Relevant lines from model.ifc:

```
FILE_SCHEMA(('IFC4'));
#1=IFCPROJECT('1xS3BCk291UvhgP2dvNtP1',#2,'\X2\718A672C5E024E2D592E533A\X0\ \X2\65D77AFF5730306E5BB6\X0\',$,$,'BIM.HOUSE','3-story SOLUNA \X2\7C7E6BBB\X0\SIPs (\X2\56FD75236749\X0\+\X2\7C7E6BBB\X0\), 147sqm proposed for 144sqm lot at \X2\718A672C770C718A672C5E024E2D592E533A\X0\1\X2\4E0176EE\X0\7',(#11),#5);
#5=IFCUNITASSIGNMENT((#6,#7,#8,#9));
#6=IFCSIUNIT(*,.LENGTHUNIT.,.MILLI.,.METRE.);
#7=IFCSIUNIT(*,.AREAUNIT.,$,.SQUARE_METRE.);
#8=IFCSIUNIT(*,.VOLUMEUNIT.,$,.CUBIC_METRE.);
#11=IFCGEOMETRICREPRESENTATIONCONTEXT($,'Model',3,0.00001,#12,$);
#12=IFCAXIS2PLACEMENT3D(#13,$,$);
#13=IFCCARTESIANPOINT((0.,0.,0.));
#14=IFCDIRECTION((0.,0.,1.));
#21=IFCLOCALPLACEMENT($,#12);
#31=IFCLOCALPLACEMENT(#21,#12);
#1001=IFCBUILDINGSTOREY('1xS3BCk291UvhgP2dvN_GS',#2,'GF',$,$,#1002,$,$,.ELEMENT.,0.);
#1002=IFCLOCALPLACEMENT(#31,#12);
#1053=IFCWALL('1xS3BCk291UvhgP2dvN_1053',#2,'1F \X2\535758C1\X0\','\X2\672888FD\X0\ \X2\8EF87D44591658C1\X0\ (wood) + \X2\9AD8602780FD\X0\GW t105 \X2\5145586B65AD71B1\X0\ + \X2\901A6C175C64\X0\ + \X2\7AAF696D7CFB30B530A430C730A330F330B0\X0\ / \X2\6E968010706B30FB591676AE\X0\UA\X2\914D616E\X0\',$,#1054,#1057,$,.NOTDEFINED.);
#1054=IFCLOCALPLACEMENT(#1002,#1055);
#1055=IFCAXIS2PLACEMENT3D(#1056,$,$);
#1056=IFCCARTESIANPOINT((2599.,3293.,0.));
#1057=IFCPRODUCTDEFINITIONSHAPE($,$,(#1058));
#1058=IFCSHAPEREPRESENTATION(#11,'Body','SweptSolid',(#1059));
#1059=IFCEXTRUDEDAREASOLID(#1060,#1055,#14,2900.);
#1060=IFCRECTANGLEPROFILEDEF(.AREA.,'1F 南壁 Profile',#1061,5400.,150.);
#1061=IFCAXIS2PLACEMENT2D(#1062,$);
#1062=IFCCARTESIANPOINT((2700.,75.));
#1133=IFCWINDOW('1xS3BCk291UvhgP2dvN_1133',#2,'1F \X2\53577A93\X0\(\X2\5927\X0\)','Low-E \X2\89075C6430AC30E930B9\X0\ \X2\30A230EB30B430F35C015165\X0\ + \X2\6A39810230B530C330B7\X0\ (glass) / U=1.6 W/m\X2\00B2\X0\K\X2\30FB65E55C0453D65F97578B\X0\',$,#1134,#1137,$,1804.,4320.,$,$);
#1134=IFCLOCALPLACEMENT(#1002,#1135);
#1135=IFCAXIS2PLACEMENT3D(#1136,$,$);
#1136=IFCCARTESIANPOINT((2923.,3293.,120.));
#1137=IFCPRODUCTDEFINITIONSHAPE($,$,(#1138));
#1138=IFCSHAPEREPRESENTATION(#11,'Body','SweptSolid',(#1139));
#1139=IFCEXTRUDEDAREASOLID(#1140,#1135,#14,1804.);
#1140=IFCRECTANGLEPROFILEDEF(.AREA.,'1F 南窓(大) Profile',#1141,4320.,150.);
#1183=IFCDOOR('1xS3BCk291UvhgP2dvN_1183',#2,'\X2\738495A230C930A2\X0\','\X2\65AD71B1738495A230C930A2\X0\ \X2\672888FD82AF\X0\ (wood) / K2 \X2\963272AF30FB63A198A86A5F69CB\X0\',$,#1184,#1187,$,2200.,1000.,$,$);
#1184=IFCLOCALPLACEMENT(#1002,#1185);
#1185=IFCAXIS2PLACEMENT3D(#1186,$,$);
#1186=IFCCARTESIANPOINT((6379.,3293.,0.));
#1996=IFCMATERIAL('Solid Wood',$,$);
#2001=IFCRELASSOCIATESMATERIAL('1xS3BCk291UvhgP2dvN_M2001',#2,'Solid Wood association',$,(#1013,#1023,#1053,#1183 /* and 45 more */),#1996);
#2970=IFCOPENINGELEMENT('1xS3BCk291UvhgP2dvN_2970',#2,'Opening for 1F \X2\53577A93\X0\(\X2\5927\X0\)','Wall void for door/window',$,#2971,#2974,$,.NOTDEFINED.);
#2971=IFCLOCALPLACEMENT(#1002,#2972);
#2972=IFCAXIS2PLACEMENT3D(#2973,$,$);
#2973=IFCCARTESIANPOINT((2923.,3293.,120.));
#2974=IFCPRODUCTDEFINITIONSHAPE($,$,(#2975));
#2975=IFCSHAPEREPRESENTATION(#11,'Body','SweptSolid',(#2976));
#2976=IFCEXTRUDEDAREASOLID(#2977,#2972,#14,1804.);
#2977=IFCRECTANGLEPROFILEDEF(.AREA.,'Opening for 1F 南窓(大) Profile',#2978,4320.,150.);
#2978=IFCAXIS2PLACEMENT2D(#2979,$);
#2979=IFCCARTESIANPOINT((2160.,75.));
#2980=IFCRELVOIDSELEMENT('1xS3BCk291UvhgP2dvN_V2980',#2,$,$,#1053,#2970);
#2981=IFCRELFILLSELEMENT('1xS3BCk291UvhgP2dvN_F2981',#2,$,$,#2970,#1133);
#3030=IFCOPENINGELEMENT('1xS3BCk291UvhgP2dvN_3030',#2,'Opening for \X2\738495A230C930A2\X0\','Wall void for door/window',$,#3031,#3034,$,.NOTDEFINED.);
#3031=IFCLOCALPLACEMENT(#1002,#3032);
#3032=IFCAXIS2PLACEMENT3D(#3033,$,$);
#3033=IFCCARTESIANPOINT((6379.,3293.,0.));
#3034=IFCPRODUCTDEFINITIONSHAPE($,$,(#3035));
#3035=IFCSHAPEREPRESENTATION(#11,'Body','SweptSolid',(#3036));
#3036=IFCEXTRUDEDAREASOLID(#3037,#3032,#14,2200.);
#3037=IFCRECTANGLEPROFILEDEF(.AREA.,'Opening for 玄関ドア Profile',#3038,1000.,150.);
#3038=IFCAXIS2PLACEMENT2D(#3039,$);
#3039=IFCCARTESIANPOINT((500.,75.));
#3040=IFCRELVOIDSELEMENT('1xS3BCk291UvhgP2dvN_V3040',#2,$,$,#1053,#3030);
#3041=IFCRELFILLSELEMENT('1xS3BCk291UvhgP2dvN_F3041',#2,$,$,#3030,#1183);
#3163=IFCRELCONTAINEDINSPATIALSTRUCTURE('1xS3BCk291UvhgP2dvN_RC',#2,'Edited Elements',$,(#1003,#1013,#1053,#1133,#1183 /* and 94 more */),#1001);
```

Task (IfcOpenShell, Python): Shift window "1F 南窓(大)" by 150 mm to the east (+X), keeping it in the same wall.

```python
import ifcopenshell
import ifcopenshell.api.geometry
import ifcopenshell.util.placement
import ifcopenshell.util.unit

model = ifcopenshell.open("model.ifc")
unit_scale = ifcopenshell.util.unit.calculate_unit_scale(model)

window = model.by_guid("1xS3BCk291UvhgP2dvN_1133")
opening = window.FillsVoids[0].RelatingOpeningElement
wall = opening.VoidsElements[0].RelatingBuildingElement

wall_matrix = ifcopenshell.util.placement.get_local_placement(wall.ObjectPlacement)
shift = wall_matrix[:3, 0] * 0.15 / unit_scale
before = ifcopenshell.util.placement.get_local_placement(window.ObjectPlacement)[:3, 3].copy()

# The window is not placed relative to its opening, so move both.
for product in (opening, window):
    matrix = ifcopenshell.util.placement.get_local_placement(product.ObjectPlacement)
    matrix[:3, 3] += shift
    ifcopenshell.api.geometry.edit_object_placement(model, product=product, matrix=matrix, is_si=False)

after = ifcopenshell.util.placement.get_local_placement(window.ObjectPlacement)[:3, 3]
print("window moved by", (after - before).round(3) + 0.0)

model.write("model_edited.ifc")
```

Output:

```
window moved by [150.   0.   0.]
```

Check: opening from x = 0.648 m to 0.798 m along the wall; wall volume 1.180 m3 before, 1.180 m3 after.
